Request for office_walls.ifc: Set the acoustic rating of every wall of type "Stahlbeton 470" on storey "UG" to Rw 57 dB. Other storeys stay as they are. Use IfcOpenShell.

First a look at what the model holds.

```python
import ifcopenshell
import ifcopenshell.util.element

model = ifcopenshell.open("office_walls.ifc")
print(model.schema)
storey = next(s for s in model.by_type("IfcBuildingStorey") if s.Name == "UG")
walls = [e for e in ifcopenshell.util.element.get_decomposition(storey) if e.is_a("IfcWall")]
seen = {}
for e in walls:
    element_type = ifcopenshell.util.element.get_type(e)
    key = (element_type.Name if element_type != e and element_type else None, ifcopenshell.util.element.get_pset(e, "Pset_WallCommon", "AcousticRating"))
    seen[key] = seen.get(key, 0) + 1
for (name, value), count in sorted(seen.items(), key=str):
    print(count, "x", name, "|", value)
```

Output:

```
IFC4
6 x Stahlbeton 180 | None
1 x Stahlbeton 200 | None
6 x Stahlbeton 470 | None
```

```python
import ifcopenshell
import ifcopenshell.api.pset
import ifcopenshell.util.element

model = ifcopenshell.open("office_walls.ifc")

storey = next(s for s in model.by_type("IfcBuildingStorey") if s.Name == "UG")
walls = [e for e in ifcopenshell.util.element.get_decomposition(storey) if e.is_a("IfcWall")]

count = 0
for e in walls:
    element_type = ifcopenshell.util.element.get_type(e)
    if element_type in (None, e) or element_type.Name != "Stahlbeton 470":
        continue
    # add_pset returns the element's existing set when there is one.
    pset = ifcopenshell.api.pset.add_pset(model, product=e, name="Pset_WallCommon")
    ifcopenshell.api.pset.edit_pset(model, pset=pset, properties={"AcousticRating": "Rw 57 dB"})
    count += 1

print(count, "walls updated")

model.write("office_walls_rev.ifc")
```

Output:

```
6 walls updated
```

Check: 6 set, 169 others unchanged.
